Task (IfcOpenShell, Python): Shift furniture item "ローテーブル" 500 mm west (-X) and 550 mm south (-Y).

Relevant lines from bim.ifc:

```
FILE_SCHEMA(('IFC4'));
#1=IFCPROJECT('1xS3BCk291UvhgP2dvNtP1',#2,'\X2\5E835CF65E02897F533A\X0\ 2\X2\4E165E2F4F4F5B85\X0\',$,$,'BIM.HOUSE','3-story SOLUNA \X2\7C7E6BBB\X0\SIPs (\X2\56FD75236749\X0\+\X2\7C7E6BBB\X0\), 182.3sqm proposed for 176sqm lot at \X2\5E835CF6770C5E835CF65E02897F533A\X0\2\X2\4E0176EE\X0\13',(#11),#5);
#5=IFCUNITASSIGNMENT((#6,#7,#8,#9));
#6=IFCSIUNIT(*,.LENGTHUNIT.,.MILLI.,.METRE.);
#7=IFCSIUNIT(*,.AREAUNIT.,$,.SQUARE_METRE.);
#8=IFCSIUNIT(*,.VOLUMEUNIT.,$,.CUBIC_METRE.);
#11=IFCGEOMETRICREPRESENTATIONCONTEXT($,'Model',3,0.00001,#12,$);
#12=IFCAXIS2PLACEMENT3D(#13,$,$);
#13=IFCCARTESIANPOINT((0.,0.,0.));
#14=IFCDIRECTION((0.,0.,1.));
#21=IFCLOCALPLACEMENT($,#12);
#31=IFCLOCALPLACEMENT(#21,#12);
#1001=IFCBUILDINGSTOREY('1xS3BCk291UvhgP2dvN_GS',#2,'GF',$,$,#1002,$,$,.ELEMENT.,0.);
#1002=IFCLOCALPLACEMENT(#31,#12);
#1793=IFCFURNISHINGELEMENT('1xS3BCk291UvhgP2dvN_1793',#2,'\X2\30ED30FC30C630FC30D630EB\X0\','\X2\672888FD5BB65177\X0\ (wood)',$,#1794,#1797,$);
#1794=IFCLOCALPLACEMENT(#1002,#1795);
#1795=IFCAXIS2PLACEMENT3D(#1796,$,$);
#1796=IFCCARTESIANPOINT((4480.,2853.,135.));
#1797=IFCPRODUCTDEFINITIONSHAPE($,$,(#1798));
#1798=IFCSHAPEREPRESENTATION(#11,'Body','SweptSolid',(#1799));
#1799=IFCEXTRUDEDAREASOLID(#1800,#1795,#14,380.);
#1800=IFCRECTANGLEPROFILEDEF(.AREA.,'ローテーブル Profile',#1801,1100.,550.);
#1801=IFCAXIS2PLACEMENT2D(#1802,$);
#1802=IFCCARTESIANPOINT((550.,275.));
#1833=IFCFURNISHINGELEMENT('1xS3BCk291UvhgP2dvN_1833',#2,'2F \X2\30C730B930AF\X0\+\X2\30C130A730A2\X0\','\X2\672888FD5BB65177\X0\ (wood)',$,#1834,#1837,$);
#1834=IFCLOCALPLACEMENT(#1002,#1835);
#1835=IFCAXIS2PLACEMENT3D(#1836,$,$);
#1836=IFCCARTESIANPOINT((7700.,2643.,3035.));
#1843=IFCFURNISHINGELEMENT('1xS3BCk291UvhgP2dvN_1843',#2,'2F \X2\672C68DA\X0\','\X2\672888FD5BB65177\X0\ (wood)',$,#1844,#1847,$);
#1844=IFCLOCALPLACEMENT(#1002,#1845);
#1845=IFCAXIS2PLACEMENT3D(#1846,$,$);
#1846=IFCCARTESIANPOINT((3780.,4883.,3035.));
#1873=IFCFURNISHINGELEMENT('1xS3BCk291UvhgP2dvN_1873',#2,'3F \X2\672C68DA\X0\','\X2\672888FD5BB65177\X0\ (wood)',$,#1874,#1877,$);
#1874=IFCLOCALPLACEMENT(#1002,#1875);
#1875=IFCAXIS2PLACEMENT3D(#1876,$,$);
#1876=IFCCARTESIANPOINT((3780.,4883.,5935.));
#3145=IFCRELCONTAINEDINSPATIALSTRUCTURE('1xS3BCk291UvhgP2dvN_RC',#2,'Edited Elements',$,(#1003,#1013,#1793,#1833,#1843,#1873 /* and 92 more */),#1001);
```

```python
import ifcopenshell
import ifcopenshell.api.geometry
import ifcopenshell.util.placement

model = ifcopenshell.open("bim.ifc")

item = model.by_id(1793)
matrix = ifcopenshell.util.placement.get_local_placement(item.ObjectPlacement)
matrix[0, 3] -= 500.0
matrix[1, 3] -= 550.0
ifcopenshell.api.geometry.edit_object_placement(model, product=item, matrix=matrix, is_si=False)

print(ifcopenshell.util.placement.get_local_placement(item.ObjectPlacement).round(3) + 0.0)

model.write("bim_updated.ifc")
```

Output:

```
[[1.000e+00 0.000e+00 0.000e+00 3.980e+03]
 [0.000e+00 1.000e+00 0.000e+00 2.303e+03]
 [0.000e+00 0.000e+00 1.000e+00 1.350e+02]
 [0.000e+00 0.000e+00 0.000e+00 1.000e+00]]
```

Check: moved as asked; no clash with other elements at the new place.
